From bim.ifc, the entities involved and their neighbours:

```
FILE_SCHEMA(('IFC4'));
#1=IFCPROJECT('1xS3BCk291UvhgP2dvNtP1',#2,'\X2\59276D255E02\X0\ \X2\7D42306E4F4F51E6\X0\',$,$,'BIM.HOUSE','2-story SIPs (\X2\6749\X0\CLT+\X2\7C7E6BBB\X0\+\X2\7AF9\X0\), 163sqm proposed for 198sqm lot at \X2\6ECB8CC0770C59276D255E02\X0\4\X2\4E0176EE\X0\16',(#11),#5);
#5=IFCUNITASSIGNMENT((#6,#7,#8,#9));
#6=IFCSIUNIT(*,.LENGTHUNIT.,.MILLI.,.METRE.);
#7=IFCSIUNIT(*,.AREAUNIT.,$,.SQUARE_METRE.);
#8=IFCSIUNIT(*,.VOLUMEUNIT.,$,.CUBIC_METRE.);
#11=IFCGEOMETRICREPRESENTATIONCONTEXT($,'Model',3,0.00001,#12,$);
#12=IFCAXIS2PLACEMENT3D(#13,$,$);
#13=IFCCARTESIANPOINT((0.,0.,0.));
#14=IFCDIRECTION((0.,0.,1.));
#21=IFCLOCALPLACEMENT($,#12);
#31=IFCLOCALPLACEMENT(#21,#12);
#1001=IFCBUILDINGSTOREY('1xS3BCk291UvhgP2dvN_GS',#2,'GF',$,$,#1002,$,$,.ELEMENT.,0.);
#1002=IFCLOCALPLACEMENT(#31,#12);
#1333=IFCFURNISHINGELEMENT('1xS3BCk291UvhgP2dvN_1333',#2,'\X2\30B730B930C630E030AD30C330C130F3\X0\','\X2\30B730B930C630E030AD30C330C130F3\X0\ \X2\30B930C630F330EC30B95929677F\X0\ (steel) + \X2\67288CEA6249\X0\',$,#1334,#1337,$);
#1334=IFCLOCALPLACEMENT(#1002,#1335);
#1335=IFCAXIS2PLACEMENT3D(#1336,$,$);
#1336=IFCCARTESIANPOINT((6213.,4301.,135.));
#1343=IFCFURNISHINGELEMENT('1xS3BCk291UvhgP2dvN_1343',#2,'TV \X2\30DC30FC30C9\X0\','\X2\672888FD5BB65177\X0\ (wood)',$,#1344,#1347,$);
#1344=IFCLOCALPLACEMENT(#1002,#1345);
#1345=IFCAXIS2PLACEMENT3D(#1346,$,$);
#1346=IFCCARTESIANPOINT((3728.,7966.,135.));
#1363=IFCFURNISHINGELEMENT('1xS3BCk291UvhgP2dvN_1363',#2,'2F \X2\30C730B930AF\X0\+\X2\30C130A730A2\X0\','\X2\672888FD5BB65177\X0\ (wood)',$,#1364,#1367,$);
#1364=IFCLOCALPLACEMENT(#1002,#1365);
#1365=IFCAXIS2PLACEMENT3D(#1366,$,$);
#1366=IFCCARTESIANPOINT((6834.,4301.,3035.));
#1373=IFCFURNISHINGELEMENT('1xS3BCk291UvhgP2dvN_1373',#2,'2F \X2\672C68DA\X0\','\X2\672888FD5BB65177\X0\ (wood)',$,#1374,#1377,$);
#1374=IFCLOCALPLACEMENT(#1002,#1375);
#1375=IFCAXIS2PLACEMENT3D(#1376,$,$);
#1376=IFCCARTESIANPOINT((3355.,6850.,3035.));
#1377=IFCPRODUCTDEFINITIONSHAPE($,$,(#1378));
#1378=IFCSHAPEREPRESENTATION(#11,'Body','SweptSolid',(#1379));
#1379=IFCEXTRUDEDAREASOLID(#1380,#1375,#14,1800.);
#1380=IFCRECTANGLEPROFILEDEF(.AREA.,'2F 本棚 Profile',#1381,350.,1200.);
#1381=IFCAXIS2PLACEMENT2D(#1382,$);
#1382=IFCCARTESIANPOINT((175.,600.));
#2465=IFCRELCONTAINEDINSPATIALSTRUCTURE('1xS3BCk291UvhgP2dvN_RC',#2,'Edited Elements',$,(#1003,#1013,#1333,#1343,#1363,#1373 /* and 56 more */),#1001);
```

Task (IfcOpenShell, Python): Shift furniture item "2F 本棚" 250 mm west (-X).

```python
import ifcopenshell
import ifcopenshell.api.geometry
import ifcopenshell.util.placement

model = ifcopenshell.open("bim.ifc")

item = model.by_guid("1xS3BCk291UvhgP2dvN_1373")
matrix = ifcopenshell.util.placement.get_local_placement(item.ObjectPlacement)
matrix[0, 3] -= 250.0
ifcopenshell.api.geometry.edit_object_placement(model, product=item, matrix=matrix, is_si=False)

print(ifcopenshell.util.placement.get_local_placement(item.ObjectPlacement).round(3) + 0.0)

model.write("bim_updated.ifc")
```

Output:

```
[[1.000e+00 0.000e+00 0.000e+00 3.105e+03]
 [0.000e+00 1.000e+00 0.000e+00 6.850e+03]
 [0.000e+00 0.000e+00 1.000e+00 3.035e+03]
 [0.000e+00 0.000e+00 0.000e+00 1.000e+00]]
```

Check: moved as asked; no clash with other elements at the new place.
